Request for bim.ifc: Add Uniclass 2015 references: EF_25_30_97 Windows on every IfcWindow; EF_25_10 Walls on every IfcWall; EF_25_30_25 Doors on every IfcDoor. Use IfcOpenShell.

First a look at what the model holds.

```python
import ifcopenshell

model = ifcopenshell.open("bim.ifc")
print(model.schema)
print("classifications:", [c.Name for c in model.by_type("IfcClassification")])
for ifc_class in ("IfcDoor", "IfcRoof", "IfcStair", "IfcWall", "IfcWindow"):
    print(ifc_class, len(model.by_type(ifc_class)))
```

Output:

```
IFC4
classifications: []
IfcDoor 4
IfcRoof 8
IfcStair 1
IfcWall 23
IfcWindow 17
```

```python
import ifcopenshell
import ifcopenshell.api.classification

model = ifcopenshell.open("bim.ifc")

system = ifcopenshell.api.classification.add_classification(model, classification="Uniclass 2015")

codes = {
    "IfcWindow": ("EF_25_30_97", "Windows"),
    "IfcWall": ("EF_25_10", "Walls"),
    "IfcDoor": ("EF_25_30_25", "Doors"),
}
for ifc_class, (code, name) in codes.items():
    products = model.by_type(ifc_class)
    ifcopenshell.api.classification.add_reference(
        model, products=products, classification=system, identification=code, name=name
    )
    print(code, len(products))

model.write("bim_rev.ifc")
```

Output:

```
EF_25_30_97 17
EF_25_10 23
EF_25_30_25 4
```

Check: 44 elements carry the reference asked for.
